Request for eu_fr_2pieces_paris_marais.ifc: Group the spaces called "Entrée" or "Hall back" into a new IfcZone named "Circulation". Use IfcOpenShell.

First a look at what the model holds.

```python
import ifcopenshell

model = ifcopenshell.open("eu_fr_2pieces_paris_marais.ifc")
print(model.schema)
seen = {}
for space in model.by_type("IfcSpace"):
    seen[space.LongName] = seen.get(space.LongName, 0) + 1
for name, count in sorted(seen.items(), key=str):
    print(count, "x", name)
print("zones:", [z.Name for z in model.by_type("IfcZone")][:20])
```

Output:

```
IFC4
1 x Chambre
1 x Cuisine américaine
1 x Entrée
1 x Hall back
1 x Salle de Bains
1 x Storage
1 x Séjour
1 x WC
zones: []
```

```python
import ifcopenshell
import ifcopenshell.api.group
import ifcopenshell.api.root

model = ifcopenshell.open("eu_fr_2pieces_paris_marais.ifc")

names = {"Entrée", "Hall back"}
spaces = [s for s in model.by_type("IfcSpace") if s.LongName in names]

zone = ifcopenshell.api.root.create_entity(model, ifc_class="IfcZone", name="Circulation")
ifcopenshell.api.group.assign_group(model, products=spaces, group=zone)
print(len(spaces), "spaces in", zone.Name)

model.write("eu_fr_2pieces_paris_marais_updated.ifc")
```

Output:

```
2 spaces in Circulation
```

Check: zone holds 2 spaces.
